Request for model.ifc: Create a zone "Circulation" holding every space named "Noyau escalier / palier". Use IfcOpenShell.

First a look at what the model holds.

```python
import ifcopenshell

model = ifcopenshell.open("model.ifc")
print(model.schema)
seen = {}
for space in model.by_type("IfcSpace"):
    seen[space.LongName] = seen.get(space.LongName, 0) + 1
for name, count in sorted(seen.items(), key=str):
    print(count, "x", name)
print("zones:", [z.Name for z in model.by_type("IfcZone")][:20])
```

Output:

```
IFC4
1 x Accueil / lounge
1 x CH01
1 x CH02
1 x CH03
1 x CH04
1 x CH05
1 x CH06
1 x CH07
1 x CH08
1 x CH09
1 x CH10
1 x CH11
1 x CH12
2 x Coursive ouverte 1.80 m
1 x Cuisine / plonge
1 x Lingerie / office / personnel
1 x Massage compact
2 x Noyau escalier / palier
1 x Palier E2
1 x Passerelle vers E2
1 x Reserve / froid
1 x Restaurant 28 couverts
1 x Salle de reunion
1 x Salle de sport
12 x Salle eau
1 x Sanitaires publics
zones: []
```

```python
import ifcopenshell
import ifcopenshell.api.group
import ifcopenshell.api.root

model = ifcopenshell.open("model.ifc")

names = {"Noyau escalier / palier"}
spaces = [s for s in model.by_type("IfcSpace") if s.LongName in names]

zone = ifcopenshell.api.root.create_entity(model, ifc_class="IfcZone", name="Circulation")
ifcopenshell.api.group.assign_group(model, products=spaces, group=zone)
print(len(spaces), "spaces in", zone.Name)

model.write("model_updated.ifc")
```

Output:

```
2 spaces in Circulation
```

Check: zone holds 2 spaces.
